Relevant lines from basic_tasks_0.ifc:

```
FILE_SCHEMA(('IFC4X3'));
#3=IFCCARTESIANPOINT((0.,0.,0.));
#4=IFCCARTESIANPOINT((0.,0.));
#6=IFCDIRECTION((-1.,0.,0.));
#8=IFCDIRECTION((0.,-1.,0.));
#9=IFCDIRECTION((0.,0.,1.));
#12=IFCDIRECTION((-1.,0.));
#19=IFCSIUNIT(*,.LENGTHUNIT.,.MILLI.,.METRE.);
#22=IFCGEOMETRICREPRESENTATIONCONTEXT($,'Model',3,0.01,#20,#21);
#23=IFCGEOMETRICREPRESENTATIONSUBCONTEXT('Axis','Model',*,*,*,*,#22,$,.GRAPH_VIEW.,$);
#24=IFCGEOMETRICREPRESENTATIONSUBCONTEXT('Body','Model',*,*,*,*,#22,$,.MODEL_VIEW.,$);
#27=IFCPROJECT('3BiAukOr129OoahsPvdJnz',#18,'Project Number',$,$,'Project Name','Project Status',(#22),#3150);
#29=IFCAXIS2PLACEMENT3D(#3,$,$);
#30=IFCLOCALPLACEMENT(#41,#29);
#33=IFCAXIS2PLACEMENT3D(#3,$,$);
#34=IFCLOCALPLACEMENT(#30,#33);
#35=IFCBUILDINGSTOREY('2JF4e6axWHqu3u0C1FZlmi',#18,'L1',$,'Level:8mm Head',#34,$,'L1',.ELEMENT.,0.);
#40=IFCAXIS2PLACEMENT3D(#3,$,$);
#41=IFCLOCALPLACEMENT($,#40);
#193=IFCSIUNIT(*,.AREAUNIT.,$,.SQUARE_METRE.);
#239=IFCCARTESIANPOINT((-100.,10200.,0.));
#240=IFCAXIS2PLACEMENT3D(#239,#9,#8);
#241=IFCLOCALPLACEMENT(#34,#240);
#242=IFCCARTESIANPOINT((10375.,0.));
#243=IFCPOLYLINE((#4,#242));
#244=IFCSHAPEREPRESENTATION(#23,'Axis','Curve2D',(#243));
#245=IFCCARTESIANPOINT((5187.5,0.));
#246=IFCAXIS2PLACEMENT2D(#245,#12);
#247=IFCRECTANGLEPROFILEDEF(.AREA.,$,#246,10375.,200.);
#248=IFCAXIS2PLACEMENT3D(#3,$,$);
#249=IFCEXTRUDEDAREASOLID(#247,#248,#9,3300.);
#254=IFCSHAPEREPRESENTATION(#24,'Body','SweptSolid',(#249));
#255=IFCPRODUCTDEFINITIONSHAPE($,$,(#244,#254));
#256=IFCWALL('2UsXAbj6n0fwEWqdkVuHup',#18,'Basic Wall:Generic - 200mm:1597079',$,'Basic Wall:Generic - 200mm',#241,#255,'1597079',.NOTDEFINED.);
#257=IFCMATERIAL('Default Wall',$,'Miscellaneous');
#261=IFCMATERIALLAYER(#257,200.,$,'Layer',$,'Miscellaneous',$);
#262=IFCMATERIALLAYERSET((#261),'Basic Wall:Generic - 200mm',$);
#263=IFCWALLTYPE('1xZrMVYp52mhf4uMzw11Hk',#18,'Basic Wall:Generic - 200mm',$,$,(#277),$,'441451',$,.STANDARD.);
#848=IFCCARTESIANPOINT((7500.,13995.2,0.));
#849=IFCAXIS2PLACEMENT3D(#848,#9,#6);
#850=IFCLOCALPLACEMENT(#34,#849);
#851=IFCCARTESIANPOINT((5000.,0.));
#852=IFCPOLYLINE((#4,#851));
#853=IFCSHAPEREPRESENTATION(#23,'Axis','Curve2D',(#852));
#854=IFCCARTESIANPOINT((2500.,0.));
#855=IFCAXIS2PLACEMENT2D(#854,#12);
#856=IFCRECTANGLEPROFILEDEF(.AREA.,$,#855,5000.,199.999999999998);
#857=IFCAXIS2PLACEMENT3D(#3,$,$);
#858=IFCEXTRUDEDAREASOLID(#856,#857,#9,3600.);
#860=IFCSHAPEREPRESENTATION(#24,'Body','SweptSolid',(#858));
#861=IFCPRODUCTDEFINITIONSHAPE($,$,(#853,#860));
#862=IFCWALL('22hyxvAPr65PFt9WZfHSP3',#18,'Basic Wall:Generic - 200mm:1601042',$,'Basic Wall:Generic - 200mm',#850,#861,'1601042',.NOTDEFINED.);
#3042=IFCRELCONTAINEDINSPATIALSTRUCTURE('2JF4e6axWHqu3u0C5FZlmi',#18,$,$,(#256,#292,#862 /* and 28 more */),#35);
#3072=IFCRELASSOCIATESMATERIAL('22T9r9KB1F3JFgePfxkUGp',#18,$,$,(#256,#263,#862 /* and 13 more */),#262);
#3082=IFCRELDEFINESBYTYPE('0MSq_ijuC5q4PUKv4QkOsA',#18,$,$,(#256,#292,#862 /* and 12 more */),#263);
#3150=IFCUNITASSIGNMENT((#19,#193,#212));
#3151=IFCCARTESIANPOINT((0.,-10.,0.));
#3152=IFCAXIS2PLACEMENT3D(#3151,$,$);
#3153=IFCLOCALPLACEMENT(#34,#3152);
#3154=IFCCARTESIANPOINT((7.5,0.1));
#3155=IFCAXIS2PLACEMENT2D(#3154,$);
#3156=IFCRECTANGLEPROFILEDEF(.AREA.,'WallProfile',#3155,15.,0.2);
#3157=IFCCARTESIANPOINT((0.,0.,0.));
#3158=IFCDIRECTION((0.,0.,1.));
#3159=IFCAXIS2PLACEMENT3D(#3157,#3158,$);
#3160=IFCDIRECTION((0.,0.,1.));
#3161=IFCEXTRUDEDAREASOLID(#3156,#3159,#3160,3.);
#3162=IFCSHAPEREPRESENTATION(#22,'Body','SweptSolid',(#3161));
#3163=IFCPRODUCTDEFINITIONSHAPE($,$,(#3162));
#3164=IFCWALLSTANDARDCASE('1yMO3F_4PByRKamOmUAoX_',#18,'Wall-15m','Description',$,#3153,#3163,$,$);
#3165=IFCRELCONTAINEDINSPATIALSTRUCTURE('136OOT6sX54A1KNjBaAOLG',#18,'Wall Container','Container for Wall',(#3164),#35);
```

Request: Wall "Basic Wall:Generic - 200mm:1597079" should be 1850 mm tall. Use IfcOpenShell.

```python
import ifcopenshell
import ifcopenshell.geom
import ifcopenshell.util.representation
import ifcopenshell.util.shape
import ifcopenshell.util.unit

model = ifcopenshell.open("basic_tasks_0.ifc")
unit_scale = ifcopenshell.util.unit.calculate_unit_scale(model)
settings = ifcopenshell.geom.settings()


def volume(element):
    """Net volume in cubic metres, openings subtracted."""
    shape = ifcopenshell.geom.create_shape(settings, element)
    return ifcopenshell.util.shape.get_volume(shape.geometry)


wall = model.by_guid("2UsXAbj6n0fwEWqdkVuHup")
before = volume(wall)

body = ifcopenshell.util.representation.get_representation(wall, "Model", "Body")
solid = body.Items[0]
old_height = solid.Depth
solid.Depth = 1.85 / unit_scale
after = volume(wall)

print(f"height {old_height:g} -> {solid.Depth:g}, volume {before:.3f} -> {after:.3f} m3")

model.write("basic_tasks_0_updated.ifc")
```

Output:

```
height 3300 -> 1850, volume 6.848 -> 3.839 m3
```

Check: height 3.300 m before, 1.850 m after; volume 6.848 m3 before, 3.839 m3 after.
